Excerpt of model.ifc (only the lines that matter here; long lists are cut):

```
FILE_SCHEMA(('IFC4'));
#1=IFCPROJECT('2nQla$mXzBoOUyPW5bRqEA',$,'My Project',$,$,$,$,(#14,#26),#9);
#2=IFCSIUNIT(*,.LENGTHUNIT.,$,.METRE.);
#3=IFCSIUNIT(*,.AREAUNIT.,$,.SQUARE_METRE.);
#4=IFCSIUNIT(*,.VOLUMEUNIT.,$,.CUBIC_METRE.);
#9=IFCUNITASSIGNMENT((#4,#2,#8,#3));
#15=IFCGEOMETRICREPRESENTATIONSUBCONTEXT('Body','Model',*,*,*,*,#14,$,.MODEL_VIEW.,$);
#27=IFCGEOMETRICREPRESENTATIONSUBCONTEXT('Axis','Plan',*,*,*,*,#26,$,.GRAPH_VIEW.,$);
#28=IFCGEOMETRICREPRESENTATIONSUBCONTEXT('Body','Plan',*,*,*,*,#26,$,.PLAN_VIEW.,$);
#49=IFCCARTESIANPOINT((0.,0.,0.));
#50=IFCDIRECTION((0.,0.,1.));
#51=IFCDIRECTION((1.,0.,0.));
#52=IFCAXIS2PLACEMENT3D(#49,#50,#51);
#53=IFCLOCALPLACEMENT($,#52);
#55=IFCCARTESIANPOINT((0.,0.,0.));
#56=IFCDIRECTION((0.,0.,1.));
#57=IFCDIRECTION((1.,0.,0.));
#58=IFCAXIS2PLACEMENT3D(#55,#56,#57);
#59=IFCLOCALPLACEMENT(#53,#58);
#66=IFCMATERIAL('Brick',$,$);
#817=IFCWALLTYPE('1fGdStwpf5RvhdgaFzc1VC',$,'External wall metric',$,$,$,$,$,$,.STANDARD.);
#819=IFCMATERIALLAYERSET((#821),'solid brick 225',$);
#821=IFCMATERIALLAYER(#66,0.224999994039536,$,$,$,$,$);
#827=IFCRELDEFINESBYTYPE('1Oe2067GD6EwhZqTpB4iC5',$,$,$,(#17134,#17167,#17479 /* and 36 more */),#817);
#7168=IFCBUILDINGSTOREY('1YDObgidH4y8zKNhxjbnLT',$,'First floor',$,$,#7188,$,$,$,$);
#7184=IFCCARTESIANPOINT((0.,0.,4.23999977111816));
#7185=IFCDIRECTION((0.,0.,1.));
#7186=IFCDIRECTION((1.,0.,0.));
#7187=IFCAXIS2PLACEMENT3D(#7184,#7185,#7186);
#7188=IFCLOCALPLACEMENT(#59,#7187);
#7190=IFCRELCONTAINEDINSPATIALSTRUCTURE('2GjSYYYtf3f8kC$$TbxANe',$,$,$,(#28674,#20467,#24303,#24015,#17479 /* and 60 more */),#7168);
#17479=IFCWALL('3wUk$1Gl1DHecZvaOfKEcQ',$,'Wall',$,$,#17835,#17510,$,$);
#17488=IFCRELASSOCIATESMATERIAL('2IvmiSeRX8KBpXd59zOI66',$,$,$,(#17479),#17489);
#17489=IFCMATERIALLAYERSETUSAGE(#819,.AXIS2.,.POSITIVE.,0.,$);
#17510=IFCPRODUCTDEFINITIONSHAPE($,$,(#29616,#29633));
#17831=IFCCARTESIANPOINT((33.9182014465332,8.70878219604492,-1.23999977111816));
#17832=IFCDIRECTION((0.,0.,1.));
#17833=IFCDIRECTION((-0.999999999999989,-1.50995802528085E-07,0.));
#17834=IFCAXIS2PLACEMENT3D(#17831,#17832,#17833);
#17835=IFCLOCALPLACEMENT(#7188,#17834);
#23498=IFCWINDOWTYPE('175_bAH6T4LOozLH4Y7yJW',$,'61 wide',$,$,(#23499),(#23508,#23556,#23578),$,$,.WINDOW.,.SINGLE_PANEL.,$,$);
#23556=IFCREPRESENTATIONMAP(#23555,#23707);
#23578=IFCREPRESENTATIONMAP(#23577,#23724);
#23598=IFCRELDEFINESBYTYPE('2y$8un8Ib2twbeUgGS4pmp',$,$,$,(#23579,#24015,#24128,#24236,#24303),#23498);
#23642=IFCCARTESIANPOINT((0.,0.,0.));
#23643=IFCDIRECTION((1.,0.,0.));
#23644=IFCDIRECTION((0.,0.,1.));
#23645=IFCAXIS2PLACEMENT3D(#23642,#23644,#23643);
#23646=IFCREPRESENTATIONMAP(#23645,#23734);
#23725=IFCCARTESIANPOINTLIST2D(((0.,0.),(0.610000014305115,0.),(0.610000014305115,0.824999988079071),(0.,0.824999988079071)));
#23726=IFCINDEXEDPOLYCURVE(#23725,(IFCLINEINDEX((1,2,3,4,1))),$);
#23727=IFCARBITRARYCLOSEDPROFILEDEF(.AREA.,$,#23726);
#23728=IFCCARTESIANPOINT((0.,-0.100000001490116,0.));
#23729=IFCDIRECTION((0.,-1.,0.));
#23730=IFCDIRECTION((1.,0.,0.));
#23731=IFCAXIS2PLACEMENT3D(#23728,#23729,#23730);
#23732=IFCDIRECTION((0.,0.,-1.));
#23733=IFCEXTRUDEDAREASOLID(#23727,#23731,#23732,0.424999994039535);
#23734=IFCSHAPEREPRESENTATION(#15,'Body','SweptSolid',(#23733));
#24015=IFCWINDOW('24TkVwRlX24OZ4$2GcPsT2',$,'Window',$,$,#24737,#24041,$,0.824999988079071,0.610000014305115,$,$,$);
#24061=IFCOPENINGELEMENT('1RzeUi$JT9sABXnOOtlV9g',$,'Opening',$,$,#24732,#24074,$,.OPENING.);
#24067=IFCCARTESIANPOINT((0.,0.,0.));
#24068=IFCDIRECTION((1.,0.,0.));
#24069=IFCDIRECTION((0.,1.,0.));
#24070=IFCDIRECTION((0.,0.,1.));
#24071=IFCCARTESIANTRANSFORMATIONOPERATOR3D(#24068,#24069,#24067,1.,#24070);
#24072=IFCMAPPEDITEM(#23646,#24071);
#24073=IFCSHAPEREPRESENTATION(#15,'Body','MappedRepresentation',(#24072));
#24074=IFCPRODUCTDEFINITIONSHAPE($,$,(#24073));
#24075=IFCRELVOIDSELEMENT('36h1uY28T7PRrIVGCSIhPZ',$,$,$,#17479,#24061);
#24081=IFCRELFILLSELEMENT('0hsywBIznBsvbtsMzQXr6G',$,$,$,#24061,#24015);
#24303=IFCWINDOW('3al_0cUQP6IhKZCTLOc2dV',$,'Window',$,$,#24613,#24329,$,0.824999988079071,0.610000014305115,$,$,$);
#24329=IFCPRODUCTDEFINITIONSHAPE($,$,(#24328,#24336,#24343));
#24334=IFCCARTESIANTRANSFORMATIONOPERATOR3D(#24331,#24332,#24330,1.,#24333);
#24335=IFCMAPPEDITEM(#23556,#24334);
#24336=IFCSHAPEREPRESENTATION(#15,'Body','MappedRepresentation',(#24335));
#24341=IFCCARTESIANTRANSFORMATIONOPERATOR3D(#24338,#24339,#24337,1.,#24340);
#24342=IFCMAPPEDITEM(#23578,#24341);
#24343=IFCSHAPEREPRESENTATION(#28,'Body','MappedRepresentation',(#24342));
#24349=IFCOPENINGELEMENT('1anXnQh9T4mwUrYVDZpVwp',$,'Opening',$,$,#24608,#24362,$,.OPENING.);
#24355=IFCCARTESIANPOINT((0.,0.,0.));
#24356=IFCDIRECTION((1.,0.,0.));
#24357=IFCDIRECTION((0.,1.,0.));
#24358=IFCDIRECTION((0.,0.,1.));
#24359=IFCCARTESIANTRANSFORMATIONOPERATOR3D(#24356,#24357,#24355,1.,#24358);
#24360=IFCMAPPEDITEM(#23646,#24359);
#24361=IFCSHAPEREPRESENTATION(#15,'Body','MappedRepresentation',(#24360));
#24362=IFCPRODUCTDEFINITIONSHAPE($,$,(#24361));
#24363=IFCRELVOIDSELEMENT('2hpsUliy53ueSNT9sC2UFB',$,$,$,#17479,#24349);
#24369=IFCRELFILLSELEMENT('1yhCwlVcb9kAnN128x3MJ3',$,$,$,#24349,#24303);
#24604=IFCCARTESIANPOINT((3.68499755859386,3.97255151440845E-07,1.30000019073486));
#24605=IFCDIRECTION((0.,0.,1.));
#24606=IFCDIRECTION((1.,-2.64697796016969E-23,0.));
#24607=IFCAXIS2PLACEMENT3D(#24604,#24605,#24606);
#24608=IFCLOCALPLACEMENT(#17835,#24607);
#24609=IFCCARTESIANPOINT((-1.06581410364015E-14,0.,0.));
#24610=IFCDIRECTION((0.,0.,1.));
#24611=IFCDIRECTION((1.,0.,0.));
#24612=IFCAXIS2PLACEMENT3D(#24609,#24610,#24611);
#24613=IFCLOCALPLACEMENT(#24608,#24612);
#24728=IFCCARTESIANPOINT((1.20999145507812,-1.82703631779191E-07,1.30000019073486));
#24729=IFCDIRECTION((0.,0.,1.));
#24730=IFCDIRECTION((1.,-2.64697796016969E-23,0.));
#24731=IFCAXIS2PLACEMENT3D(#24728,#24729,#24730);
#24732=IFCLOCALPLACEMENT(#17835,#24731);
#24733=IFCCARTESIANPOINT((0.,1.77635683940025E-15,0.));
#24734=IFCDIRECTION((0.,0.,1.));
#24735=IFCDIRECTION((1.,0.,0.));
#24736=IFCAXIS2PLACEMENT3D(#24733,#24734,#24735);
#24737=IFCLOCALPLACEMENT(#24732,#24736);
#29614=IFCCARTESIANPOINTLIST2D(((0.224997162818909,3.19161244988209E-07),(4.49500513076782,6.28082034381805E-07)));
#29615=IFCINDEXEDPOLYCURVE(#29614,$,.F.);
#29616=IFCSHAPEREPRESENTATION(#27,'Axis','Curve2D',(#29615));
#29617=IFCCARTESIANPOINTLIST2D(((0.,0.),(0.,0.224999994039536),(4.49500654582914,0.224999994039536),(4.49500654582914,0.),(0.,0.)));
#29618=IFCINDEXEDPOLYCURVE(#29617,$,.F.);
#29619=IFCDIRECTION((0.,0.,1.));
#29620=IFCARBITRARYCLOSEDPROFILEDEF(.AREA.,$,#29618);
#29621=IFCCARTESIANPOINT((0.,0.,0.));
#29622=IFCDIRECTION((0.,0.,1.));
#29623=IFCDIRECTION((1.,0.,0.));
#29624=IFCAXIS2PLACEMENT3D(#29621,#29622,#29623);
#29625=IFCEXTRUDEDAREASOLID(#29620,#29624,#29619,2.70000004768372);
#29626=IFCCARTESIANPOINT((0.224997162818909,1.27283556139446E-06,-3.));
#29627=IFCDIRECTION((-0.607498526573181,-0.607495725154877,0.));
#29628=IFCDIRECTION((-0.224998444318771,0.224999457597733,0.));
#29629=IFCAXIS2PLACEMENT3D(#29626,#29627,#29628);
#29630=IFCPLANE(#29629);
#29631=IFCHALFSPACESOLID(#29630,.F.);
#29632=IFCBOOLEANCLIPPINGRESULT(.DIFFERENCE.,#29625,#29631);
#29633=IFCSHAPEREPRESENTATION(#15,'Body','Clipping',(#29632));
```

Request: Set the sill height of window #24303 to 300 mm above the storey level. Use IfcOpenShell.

```python
import numpy as np
import ifcopenshell
import ifcopenshell.api.geometry
import ifcopenshell.geom
import ifcopenshell.util.element
import ifcopenshell.util.placement
import ifcopenshell.util.shape
import ifcopenshell.util.unit

model = ifcopenshell.open("model.ifc")
unit_scale = ifcopenshell.util.unit.calculate_unit_scale(model)

window = model.by_guid("3al_0cUQP6IhKZCTLOc2dV")
opening = window.FillsVoids[0].RelatingOpeningElement
storey = ifcopenshell.util.element.get_container(window, ifc_class="IfcBuildingStorey")
level = ifcopenshell.util.placement.get_local_placement(storey.ObjectPlacement)[2, 3]

# The opening's origin need not be at the sill, so measure its lowest point.
shape = ifcopenshell.geom.create_shape(ifcopenshell.geom.settings(), opening)
bottom = ifcopenshell.util.shape.get_shape_bottom_elevation(shape, shape.geometry) / unit_scale
dz = level + 0.3 / unit_scale - bottom

shift = np.array([0.0, 0.0, dz])
# The window is placed relative to its opening, so it follows when the opening moves.
matrix = ifcopenshell.util.placement.get_local_placement(opening.ObjectPlacement)
matrix[:3, 3] += shift
ifcopenshell.api.geometry.edit_object_placement(
    model, product=opening, matrix=matrix, is_si=False, should_transform_children=True
)

print(f"moved by {dz * unit_scale:+.3f} m")

model.write("model_rev.ifc")
```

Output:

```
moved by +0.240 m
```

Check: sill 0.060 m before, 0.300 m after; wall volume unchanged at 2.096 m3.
